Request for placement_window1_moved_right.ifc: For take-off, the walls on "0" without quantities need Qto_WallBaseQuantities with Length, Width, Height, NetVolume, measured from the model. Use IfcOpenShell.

First a look at what the model holds.

```python
import ifcopenshell
import ifcopenshell.util.element
import ifcopenshell.util.unit

model = ifcopenshell.open("placement_window1_moved_right.ifc")
print(model.schema)
for unit_type in ("LENGTHUNIT", "AREAUNIT", "VOLUMEUNIT"):
    print(unit_type, ifcopenshell.util.unit.calculate_unit_scale(model, unit_type))
storey = next(s for s in model.by_type("IfcBuildingStorey") if s.Name == "0")
walls = [e for e in ifcopenshell.util.element.get_decomposition(storey) if e.is_a("IfcWall")]
for e in sorted(walls, key=lambda e: e.id()):
    print(e.id(), e.is_a(), e.Name, list(ifcopenshell.util.element.get_psets(e, qtos_only=True)), sep=" | ")
```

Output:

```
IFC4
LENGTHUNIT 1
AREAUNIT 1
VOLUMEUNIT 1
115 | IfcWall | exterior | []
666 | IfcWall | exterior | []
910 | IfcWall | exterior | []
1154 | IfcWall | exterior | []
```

```python
import ifcopenshell
import ifcopenshell.api.pset
import ifcopenshell.geom
import ifcopenshell.util.element
import ifcopenshell.util.shape
import ifcopenshell.util.unit

model = ifcopenshell.open("placement_window1_moved_right.ifc")
unit_scale = ifcopenshell.util.unit.calculate_unit_scale(model)
volume_scale = ifcopenshell.util.unit.calculate_unit_scale(model, "VOLUMEUNIT")
settings = ifcopenshell.geom.settings()

storey = next(s for s in model.by_type("IfcBuildingStorey") if s.Name == "0")
walls = [e for e in ifcopenshell.util.element.get_decomposition(storey) if e.is_a("IfcWall")]

for e in sorted(walls, key=lambda e: e.id()):
    if ifcopenshell.util.element.get_psets(e, qtos_only=True, should_inherit=False):
        continue
    # Geometry comes back in metres, in the element's own axes.
    shape = ifcopenshell.geom.create_shape(settings, e)
    values = {
        "Length": ifcopenshell.util.shape.get_x(shape.geometry) / unit_scale,
        "Width": ifcopenshell.util.shape.get_y(shape.geometry) / unit_scale,
        "Height": ifcopenshell.util.shape.get_z(shape.geometry) / unit_scale,
        "NetVolume": ifcopenshell.util.shape.get_volume(shape.geometry) / volume_scale,
    }
    qto = ifcopenshell.api.pset.add_qto(model, product=e, name="Qto_WallBaseQuantities")
    ifcopenshell.api.pset.edit_qto(model, qto=qto, properties=values)
    print(e.id(), {k: round(v, 3) for k, v in values.items()})

model.write("placement_window1_moved_right_rev.ifc")
```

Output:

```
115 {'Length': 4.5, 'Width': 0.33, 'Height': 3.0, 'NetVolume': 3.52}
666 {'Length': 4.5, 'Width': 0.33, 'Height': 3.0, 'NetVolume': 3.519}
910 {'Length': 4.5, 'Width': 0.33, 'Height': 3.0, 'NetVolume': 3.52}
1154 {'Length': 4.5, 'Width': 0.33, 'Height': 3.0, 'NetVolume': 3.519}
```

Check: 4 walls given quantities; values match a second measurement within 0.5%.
